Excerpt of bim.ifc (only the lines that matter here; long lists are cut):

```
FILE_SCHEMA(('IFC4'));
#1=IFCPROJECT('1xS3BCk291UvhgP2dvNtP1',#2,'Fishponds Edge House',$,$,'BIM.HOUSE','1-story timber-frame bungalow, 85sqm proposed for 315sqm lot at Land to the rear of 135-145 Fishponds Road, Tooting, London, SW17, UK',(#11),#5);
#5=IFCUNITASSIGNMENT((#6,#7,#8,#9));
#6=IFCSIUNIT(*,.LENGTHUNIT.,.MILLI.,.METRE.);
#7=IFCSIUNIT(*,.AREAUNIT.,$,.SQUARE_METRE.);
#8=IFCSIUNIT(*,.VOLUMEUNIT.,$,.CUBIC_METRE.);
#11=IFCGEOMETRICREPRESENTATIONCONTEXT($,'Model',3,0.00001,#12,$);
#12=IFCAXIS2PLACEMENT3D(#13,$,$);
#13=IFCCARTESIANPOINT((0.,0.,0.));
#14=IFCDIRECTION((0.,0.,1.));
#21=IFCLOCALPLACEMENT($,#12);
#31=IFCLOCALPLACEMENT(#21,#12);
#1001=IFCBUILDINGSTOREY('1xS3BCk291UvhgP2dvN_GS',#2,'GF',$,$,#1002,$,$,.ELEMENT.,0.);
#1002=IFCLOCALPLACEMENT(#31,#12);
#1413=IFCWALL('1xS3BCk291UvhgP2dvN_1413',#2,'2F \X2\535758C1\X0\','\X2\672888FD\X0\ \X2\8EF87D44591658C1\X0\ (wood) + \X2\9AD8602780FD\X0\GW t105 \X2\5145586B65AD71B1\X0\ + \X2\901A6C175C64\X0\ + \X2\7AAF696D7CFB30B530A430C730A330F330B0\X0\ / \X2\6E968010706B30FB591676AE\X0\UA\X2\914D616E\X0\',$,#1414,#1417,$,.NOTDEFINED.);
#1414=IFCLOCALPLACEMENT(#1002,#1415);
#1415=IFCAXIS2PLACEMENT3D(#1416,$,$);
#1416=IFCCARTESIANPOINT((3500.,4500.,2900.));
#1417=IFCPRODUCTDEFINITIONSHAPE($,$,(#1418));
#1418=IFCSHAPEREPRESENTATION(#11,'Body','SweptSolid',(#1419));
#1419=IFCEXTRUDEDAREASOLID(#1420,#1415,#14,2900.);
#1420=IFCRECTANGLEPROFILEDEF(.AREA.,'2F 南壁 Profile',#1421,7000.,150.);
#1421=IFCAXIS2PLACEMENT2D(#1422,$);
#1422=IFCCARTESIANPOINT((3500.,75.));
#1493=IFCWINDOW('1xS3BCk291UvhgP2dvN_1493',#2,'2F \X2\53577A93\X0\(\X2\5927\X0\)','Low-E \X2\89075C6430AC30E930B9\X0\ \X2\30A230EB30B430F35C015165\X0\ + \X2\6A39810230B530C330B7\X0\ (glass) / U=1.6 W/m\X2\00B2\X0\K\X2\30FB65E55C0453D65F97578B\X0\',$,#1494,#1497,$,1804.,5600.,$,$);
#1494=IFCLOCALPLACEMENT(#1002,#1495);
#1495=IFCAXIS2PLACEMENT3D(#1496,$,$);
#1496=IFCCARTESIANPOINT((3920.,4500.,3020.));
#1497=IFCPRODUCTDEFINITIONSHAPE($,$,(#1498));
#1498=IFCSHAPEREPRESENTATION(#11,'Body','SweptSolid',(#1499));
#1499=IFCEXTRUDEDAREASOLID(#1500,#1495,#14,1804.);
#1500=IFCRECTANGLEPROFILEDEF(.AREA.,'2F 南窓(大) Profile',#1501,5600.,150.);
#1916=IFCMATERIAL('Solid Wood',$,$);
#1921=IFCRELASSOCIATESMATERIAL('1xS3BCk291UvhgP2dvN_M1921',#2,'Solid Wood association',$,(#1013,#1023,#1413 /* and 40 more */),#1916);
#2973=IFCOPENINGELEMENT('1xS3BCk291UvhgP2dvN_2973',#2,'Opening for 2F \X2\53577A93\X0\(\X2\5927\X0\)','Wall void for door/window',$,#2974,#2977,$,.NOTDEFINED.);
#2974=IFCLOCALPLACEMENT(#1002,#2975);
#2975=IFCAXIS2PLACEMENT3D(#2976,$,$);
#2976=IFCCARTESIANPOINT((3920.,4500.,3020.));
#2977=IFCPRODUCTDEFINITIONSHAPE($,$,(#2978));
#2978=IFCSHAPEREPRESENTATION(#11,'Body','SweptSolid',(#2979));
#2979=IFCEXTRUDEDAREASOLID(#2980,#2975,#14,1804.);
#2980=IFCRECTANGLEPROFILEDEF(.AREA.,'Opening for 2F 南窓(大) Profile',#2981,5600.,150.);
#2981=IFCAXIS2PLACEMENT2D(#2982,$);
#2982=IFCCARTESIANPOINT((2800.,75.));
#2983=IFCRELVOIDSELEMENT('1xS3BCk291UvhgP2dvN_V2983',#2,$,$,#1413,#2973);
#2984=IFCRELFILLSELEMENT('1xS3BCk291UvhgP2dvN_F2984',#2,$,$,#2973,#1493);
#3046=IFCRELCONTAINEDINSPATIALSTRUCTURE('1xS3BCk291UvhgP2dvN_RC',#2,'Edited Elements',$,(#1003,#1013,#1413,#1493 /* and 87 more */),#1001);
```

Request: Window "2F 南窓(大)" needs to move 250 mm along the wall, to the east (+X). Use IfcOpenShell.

```python
import ifcopenshell
import ifcopenshell.api.geometry
import ifcopenshell.util.placement
import ifcopenshell.util.unit

model = ifcopenshell.open("bim.ifc")
unit_scale = ifcopenshell.util.unit.calculate_unit_scale(model)

window = model.by_guid("1xS3BCk291UvhgP2dvN_1493")
opening = window.FillsVoids[0].RelatingOpeningElement
wall = opening.VoidsElements[0].RelatingBuildingElement

wall_matrix = ifcopenshell.util.placement.get_local_placement(wall.ObjectPlacement)
shift = wall_matrix[:3, 0] * 0.25 / unit_scale
before = ifcopenshell.util.placement.get_local_placement(window.ObjectPlacement)[:3, 3].copy()

# The window is not placed relative to its opening, so move both.
for product in (opening, window):
    matrix = ifcopenshell.util.placement.get_local_placement(product.ObjectPlacement)
    matrix[:3, 3] += shift
    ifcopenshell.api.geometry.edit_object_placement(model, product=product, matrix=matrix, is_si=False)

after = ifcopenshell.util.placement.get_local_placement(window.ObjectPlacement)[:3, 3]
print("window moved by", (after - before).round(3) + 0.0)

model.write("bim_updated.ifc")
```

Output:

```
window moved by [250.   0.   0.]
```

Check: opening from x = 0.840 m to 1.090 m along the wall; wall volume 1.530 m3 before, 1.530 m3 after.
